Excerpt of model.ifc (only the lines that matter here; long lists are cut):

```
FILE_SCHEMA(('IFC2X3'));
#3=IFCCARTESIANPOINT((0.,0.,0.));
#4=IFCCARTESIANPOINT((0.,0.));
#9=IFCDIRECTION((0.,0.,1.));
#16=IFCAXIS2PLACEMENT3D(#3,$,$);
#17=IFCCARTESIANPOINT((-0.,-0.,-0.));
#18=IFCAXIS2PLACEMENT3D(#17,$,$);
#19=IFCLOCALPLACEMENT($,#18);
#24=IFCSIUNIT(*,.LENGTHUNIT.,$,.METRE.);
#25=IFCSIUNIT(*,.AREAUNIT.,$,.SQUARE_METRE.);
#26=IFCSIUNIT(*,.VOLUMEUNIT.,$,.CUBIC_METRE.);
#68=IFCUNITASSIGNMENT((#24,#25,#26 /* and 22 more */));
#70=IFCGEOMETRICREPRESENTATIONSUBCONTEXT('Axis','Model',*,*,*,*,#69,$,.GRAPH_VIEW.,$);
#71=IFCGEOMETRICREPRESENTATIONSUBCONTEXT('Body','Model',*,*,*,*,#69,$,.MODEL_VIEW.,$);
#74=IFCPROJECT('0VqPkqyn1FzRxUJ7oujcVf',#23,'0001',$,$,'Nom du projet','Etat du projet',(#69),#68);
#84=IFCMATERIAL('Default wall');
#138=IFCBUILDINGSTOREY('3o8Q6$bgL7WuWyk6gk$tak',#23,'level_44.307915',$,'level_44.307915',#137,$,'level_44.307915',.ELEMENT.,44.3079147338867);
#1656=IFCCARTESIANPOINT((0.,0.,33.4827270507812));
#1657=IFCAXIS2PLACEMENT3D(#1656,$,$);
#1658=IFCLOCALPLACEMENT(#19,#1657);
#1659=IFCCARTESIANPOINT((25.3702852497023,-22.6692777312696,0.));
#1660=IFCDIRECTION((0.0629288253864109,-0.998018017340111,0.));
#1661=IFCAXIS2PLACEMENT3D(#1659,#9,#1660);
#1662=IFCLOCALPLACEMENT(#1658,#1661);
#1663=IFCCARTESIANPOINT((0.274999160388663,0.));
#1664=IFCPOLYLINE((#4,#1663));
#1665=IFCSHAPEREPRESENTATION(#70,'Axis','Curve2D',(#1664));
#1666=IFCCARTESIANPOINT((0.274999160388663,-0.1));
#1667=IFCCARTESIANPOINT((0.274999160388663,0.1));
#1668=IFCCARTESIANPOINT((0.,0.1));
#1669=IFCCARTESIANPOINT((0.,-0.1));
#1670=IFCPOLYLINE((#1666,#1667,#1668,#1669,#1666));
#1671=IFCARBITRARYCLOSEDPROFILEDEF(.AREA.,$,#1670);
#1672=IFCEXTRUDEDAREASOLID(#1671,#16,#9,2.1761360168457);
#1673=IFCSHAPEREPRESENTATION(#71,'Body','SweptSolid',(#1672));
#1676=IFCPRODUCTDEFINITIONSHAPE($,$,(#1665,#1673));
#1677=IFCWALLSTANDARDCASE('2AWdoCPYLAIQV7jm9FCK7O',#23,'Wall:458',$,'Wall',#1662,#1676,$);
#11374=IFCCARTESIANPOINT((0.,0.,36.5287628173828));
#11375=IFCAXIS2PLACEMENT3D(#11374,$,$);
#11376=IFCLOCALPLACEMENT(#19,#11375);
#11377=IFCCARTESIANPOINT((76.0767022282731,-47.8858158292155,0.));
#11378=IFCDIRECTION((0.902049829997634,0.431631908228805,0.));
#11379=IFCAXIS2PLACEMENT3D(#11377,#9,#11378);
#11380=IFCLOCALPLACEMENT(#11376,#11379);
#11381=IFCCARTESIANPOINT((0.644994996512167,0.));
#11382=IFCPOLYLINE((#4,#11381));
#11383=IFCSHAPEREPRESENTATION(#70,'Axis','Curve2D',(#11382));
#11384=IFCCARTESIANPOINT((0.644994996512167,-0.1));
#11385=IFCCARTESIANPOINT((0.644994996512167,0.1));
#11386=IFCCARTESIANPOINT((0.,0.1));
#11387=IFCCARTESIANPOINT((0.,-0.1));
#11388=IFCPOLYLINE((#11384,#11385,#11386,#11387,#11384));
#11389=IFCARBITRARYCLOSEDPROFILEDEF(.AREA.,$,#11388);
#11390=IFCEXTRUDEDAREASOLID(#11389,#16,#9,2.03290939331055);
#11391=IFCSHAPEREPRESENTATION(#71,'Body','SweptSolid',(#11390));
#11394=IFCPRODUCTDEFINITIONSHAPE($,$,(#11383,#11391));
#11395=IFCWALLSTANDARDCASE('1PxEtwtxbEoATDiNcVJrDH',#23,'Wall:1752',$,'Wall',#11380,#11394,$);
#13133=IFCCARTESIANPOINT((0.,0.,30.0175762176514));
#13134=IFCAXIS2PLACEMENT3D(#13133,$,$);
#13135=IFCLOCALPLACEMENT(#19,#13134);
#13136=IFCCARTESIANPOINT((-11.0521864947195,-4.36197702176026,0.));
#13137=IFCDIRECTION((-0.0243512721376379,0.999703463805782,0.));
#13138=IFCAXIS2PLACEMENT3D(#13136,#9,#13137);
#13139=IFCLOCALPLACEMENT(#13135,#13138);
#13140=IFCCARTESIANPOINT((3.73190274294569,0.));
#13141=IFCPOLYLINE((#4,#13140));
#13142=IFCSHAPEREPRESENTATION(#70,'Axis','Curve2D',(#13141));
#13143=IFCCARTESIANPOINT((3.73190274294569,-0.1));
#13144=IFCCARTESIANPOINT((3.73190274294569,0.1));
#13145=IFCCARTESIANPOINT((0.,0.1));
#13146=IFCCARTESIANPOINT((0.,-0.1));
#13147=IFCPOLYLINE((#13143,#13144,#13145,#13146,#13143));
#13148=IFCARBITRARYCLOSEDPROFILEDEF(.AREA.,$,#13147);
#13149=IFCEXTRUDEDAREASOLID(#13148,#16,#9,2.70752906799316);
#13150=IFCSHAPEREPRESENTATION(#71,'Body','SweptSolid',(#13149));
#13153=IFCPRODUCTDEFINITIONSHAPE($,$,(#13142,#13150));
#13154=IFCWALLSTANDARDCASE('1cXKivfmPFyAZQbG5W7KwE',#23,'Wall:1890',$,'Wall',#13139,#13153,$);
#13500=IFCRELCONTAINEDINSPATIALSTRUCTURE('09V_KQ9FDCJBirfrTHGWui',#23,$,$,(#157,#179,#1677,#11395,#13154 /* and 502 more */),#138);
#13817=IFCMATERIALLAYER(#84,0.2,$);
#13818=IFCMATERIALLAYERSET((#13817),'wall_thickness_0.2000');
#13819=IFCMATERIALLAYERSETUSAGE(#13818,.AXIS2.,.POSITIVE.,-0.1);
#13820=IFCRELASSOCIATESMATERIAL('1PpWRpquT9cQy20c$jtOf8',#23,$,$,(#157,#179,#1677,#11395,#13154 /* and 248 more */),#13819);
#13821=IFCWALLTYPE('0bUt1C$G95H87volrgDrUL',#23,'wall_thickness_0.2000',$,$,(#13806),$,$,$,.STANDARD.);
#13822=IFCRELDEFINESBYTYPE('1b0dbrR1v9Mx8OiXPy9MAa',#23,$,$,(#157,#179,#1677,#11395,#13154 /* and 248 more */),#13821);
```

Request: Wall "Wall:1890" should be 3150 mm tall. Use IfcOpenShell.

```python
import ifcopenshell
import ifcopenshell.geom
import ifcopenshell.util.representation
import ifcopenshell.util.shape
import ifcopenshell.util.unit

model = ifcopenshell.open("model.ifc")
unit_scale = ifcopenshell.util.unit.calculate_unit_scale(model)
settings = ifcopenshell.geom.settings()


def volume(element):
    """Net volume in cubic metres, openings subtracted."""
    shape = ifcopenshell.geom.create_shape(settings, element)
    return ifcopenshell.util.shape.get_volume(shape.geometry)


wall = model.by_id(13154)
before = volume(wall)

body = ifcopenshell.util.representation.get_representation(wall, "Model", "Body")
solid = body.Items[0]
old_height = solid.Depth
solid.Depth = 3.15 / unit_scale
after = volume(wall)

print(f"height {old_height:g} -> {solid.Depth:g}, volume {before:.3f} -> {after:.3f} m3")

model.write("model_rev.ifc")
```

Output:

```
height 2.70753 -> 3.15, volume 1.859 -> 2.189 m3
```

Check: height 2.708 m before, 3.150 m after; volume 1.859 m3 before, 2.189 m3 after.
